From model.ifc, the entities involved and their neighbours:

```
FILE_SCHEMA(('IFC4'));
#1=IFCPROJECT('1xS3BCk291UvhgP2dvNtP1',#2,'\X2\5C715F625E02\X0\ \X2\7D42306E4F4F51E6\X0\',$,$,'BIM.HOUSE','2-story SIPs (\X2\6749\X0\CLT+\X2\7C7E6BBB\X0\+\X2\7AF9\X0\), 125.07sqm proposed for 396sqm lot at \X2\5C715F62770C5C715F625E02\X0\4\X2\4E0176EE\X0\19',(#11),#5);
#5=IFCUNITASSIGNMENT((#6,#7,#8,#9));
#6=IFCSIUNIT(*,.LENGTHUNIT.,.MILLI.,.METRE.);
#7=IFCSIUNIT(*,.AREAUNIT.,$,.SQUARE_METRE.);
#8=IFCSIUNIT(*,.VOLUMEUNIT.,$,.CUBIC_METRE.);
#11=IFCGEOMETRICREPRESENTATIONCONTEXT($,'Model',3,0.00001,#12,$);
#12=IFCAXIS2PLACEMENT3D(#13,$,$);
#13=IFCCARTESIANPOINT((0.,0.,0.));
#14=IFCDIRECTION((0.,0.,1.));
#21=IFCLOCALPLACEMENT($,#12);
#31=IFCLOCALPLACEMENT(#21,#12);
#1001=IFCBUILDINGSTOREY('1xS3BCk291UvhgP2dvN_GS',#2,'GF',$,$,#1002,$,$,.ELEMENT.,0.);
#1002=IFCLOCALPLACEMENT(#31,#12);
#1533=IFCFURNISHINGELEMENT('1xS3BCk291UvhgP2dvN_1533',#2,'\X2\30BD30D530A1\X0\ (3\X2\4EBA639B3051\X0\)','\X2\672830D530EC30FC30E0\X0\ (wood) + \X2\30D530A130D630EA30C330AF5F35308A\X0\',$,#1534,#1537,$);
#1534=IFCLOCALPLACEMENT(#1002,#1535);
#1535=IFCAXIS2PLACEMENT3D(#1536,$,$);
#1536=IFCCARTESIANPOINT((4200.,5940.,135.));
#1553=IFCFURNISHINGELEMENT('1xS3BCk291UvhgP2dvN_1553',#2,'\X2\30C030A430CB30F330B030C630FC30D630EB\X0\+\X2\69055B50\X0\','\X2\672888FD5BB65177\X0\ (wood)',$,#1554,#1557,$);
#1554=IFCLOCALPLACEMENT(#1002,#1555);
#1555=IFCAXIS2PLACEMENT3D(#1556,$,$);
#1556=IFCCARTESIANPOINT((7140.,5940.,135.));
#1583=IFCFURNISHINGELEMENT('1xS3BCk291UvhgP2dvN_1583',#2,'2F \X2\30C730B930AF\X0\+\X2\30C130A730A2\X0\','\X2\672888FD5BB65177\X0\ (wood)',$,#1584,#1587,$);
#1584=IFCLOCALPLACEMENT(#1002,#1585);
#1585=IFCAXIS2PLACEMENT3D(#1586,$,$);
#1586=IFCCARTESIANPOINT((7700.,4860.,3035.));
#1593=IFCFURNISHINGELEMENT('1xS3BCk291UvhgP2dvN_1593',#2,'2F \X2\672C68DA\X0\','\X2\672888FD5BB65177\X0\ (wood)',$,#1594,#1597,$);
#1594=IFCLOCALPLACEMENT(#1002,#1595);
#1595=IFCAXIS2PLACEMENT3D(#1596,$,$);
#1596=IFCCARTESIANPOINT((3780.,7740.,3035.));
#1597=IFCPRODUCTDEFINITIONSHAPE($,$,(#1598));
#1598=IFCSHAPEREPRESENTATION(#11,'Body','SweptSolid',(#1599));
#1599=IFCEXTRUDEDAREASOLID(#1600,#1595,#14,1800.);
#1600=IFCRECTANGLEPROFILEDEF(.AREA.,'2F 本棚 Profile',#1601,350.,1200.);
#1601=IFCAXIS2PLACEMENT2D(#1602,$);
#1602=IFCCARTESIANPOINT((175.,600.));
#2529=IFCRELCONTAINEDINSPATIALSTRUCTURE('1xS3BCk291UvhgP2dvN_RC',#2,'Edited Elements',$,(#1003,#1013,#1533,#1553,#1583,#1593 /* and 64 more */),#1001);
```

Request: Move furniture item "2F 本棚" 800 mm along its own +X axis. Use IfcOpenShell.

```python
import ifcopenshell
import ifcopenshell.api.geometry
import ifcopenshell.util.placement
import ifcopenshell.util.unit

model = ifcopenshell.open("model.ifc")
unit_scale = ifcopenshell.util.unit.calculate_unit_scale(model)

item = model.by_id(1593)
matrix = ifcopenshell.util.placement.get_local_placement(item.ObjectPlacement)
matrix[:3, 3] += matrix[:3, 0] * 0.8 / unit_scale
ifcopenshell.api.geometry.edit_object_placement(model, product=item, matrix=matrix, is_si=False)

print(ifcopenshell.util.placement.get_local_placement(item.ObjectPlacement).round(3) + 0.0)

model.write("model_rev.ifc")
```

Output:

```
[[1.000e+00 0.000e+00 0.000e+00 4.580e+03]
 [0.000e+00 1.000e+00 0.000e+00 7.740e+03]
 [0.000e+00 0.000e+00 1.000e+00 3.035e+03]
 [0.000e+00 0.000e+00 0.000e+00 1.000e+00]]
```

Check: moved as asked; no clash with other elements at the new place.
